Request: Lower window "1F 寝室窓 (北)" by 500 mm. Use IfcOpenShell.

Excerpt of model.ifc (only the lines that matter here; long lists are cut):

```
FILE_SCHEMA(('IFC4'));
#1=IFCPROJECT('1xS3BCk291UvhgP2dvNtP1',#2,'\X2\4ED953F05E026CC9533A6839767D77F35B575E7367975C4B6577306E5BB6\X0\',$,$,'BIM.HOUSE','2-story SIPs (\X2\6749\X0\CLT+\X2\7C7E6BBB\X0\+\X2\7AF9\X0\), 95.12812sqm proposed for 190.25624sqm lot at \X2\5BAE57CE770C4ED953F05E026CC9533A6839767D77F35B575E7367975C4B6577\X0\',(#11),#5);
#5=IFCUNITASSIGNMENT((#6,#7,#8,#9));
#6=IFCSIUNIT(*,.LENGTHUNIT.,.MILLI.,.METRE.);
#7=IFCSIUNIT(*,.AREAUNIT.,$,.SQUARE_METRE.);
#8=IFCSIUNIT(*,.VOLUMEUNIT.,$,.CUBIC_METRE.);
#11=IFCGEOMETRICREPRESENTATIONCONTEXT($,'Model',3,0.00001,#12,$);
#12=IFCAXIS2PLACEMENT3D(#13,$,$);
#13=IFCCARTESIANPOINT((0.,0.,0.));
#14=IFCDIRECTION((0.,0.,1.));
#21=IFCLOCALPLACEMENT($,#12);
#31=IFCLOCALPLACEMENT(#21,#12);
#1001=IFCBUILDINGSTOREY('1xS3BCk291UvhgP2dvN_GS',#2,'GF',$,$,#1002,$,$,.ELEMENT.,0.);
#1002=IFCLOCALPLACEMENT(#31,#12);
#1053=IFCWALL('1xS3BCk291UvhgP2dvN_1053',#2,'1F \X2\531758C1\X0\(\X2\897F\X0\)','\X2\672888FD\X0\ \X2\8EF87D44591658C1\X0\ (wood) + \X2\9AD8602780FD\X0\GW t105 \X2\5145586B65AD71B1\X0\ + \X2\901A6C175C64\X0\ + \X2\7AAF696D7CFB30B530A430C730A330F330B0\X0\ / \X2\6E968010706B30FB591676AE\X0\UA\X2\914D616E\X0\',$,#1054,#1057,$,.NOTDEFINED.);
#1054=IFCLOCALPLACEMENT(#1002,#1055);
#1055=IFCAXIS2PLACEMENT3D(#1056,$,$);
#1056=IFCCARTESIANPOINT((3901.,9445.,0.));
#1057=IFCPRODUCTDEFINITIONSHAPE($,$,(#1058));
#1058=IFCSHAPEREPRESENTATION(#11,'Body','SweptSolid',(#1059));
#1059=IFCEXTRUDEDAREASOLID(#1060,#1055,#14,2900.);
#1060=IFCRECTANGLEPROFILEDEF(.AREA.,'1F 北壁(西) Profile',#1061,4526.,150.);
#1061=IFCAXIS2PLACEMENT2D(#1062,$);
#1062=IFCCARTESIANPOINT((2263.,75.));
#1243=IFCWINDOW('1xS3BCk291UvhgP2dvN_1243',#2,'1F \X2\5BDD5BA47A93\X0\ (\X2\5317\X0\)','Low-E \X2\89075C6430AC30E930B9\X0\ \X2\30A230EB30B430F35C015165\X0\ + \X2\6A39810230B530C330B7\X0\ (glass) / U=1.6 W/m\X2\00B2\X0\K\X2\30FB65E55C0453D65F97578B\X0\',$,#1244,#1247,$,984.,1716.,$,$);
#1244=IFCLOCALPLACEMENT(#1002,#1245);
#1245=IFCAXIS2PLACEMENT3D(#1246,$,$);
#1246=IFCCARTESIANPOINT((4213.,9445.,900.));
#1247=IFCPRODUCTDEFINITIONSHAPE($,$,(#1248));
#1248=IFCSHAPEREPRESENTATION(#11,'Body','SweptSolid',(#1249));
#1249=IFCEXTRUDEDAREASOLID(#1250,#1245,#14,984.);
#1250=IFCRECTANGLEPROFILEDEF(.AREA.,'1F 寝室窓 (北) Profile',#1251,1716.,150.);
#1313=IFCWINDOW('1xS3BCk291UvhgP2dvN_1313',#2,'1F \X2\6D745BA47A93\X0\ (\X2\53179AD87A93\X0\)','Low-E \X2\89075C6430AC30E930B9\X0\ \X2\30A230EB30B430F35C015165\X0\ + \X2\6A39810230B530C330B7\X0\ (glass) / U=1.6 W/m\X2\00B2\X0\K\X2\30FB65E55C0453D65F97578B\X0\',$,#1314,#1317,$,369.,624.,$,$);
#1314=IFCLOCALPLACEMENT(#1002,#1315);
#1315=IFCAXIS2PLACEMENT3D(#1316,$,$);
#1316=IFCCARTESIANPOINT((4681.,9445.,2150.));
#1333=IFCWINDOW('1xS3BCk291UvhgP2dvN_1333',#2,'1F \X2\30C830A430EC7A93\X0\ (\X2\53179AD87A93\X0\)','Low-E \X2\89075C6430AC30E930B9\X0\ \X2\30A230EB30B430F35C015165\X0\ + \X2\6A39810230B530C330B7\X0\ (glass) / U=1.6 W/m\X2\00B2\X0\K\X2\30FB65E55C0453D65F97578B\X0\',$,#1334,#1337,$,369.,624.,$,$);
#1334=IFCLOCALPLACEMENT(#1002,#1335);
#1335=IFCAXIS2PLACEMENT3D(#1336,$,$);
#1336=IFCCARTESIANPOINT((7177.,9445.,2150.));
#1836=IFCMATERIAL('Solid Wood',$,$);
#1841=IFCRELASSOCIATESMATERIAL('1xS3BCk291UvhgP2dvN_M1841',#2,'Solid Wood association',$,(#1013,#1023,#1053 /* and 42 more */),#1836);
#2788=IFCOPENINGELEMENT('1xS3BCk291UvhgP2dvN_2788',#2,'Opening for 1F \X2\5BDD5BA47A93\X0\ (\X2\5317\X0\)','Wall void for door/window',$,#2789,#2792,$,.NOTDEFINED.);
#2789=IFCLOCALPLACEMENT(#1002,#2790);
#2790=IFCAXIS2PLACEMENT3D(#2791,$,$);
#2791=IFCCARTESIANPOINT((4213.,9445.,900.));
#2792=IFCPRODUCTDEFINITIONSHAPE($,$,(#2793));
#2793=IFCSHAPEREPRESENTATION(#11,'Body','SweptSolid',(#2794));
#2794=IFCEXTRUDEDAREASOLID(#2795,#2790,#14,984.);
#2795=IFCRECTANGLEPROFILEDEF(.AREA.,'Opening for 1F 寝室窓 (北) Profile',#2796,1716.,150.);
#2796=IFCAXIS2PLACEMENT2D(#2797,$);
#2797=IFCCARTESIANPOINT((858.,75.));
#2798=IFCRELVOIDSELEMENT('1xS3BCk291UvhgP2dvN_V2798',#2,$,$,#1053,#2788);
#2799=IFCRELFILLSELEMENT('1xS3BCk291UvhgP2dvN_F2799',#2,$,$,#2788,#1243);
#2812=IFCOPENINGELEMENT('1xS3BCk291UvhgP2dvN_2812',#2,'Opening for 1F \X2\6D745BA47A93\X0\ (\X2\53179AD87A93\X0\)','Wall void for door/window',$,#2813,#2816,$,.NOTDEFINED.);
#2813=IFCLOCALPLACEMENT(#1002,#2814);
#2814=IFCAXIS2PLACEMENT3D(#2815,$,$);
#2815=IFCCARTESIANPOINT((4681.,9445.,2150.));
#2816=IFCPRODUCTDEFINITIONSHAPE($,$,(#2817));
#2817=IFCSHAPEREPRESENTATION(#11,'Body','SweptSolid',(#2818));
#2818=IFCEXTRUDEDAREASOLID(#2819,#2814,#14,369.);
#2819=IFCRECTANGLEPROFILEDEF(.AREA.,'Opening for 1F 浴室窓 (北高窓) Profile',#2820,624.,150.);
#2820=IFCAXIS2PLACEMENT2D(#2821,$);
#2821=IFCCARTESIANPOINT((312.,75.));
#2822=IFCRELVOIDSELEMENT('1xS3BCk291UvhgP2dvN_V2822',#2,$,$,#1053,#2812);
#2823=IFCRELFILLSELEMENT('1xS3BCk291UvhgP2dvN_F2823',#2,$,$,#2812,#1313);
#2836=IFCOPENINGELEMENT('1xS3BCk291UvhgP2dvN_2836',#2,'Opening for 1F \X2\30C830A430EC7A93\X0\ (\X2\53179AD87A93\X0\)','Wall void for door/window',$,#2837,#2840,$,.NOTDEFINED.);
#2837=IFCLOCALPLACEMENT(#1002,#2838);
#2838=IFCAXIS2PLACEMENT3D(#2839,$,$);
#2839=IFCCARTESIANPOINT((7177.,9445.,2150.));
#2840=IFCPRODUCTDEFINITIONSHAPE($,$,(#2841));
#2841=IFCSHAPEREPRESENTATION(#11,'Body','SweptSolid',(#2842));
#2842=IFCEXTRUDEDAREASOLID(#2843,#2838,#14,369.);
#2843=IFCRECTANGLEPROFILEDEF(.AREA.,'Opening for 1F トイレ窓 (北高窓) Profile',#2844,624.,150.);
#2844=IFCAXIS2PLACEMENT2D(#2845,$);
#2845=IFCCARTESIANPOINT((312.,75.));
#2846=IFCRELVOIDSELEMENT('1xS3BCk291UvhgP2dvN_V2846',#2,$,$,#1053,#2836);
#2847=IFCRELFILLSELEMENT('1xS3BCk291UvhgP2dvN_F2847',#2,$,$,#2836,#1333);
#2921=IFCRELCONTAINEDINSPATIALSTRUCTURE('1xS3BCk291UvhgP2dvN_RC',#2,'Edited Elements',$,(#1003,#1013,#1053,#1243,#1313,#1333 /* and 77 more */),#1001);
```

```python
import numpy as np
import ifcopenshell
import ifcopenshell.api.geometry
import ifcopenshell.util.placement
import ifcopenshell.util.unit

model = ifcopenshell.open("model.ifc")
unit_scale = ifcopenshell.util.unit.calculate_unit_scale(model)

window = model.by_id(1243)
opening = window.FillsVoids[0].RelatingOpeningElement
dz = -500.0

shift = np.array([0.0, 0.0, dz])
# The window is not placed relative to its opening, so move both.
for product in (opening, window):
    matrix = ifcopenshell.util.placement.get_local_placement(product.ObjectPlacement)
    matrix[:3, 3] += shift
    ifcopenshell.api.geometry.edit_object_placement(model, product=product, matrix=matrix, is_si=False)

print(f"moved by {dz * unit_scale:+.3f} m")

model.write("model_rev.ifc")
```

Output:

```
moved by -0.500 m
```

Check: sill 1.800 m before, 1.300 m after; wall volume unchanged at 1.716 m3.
